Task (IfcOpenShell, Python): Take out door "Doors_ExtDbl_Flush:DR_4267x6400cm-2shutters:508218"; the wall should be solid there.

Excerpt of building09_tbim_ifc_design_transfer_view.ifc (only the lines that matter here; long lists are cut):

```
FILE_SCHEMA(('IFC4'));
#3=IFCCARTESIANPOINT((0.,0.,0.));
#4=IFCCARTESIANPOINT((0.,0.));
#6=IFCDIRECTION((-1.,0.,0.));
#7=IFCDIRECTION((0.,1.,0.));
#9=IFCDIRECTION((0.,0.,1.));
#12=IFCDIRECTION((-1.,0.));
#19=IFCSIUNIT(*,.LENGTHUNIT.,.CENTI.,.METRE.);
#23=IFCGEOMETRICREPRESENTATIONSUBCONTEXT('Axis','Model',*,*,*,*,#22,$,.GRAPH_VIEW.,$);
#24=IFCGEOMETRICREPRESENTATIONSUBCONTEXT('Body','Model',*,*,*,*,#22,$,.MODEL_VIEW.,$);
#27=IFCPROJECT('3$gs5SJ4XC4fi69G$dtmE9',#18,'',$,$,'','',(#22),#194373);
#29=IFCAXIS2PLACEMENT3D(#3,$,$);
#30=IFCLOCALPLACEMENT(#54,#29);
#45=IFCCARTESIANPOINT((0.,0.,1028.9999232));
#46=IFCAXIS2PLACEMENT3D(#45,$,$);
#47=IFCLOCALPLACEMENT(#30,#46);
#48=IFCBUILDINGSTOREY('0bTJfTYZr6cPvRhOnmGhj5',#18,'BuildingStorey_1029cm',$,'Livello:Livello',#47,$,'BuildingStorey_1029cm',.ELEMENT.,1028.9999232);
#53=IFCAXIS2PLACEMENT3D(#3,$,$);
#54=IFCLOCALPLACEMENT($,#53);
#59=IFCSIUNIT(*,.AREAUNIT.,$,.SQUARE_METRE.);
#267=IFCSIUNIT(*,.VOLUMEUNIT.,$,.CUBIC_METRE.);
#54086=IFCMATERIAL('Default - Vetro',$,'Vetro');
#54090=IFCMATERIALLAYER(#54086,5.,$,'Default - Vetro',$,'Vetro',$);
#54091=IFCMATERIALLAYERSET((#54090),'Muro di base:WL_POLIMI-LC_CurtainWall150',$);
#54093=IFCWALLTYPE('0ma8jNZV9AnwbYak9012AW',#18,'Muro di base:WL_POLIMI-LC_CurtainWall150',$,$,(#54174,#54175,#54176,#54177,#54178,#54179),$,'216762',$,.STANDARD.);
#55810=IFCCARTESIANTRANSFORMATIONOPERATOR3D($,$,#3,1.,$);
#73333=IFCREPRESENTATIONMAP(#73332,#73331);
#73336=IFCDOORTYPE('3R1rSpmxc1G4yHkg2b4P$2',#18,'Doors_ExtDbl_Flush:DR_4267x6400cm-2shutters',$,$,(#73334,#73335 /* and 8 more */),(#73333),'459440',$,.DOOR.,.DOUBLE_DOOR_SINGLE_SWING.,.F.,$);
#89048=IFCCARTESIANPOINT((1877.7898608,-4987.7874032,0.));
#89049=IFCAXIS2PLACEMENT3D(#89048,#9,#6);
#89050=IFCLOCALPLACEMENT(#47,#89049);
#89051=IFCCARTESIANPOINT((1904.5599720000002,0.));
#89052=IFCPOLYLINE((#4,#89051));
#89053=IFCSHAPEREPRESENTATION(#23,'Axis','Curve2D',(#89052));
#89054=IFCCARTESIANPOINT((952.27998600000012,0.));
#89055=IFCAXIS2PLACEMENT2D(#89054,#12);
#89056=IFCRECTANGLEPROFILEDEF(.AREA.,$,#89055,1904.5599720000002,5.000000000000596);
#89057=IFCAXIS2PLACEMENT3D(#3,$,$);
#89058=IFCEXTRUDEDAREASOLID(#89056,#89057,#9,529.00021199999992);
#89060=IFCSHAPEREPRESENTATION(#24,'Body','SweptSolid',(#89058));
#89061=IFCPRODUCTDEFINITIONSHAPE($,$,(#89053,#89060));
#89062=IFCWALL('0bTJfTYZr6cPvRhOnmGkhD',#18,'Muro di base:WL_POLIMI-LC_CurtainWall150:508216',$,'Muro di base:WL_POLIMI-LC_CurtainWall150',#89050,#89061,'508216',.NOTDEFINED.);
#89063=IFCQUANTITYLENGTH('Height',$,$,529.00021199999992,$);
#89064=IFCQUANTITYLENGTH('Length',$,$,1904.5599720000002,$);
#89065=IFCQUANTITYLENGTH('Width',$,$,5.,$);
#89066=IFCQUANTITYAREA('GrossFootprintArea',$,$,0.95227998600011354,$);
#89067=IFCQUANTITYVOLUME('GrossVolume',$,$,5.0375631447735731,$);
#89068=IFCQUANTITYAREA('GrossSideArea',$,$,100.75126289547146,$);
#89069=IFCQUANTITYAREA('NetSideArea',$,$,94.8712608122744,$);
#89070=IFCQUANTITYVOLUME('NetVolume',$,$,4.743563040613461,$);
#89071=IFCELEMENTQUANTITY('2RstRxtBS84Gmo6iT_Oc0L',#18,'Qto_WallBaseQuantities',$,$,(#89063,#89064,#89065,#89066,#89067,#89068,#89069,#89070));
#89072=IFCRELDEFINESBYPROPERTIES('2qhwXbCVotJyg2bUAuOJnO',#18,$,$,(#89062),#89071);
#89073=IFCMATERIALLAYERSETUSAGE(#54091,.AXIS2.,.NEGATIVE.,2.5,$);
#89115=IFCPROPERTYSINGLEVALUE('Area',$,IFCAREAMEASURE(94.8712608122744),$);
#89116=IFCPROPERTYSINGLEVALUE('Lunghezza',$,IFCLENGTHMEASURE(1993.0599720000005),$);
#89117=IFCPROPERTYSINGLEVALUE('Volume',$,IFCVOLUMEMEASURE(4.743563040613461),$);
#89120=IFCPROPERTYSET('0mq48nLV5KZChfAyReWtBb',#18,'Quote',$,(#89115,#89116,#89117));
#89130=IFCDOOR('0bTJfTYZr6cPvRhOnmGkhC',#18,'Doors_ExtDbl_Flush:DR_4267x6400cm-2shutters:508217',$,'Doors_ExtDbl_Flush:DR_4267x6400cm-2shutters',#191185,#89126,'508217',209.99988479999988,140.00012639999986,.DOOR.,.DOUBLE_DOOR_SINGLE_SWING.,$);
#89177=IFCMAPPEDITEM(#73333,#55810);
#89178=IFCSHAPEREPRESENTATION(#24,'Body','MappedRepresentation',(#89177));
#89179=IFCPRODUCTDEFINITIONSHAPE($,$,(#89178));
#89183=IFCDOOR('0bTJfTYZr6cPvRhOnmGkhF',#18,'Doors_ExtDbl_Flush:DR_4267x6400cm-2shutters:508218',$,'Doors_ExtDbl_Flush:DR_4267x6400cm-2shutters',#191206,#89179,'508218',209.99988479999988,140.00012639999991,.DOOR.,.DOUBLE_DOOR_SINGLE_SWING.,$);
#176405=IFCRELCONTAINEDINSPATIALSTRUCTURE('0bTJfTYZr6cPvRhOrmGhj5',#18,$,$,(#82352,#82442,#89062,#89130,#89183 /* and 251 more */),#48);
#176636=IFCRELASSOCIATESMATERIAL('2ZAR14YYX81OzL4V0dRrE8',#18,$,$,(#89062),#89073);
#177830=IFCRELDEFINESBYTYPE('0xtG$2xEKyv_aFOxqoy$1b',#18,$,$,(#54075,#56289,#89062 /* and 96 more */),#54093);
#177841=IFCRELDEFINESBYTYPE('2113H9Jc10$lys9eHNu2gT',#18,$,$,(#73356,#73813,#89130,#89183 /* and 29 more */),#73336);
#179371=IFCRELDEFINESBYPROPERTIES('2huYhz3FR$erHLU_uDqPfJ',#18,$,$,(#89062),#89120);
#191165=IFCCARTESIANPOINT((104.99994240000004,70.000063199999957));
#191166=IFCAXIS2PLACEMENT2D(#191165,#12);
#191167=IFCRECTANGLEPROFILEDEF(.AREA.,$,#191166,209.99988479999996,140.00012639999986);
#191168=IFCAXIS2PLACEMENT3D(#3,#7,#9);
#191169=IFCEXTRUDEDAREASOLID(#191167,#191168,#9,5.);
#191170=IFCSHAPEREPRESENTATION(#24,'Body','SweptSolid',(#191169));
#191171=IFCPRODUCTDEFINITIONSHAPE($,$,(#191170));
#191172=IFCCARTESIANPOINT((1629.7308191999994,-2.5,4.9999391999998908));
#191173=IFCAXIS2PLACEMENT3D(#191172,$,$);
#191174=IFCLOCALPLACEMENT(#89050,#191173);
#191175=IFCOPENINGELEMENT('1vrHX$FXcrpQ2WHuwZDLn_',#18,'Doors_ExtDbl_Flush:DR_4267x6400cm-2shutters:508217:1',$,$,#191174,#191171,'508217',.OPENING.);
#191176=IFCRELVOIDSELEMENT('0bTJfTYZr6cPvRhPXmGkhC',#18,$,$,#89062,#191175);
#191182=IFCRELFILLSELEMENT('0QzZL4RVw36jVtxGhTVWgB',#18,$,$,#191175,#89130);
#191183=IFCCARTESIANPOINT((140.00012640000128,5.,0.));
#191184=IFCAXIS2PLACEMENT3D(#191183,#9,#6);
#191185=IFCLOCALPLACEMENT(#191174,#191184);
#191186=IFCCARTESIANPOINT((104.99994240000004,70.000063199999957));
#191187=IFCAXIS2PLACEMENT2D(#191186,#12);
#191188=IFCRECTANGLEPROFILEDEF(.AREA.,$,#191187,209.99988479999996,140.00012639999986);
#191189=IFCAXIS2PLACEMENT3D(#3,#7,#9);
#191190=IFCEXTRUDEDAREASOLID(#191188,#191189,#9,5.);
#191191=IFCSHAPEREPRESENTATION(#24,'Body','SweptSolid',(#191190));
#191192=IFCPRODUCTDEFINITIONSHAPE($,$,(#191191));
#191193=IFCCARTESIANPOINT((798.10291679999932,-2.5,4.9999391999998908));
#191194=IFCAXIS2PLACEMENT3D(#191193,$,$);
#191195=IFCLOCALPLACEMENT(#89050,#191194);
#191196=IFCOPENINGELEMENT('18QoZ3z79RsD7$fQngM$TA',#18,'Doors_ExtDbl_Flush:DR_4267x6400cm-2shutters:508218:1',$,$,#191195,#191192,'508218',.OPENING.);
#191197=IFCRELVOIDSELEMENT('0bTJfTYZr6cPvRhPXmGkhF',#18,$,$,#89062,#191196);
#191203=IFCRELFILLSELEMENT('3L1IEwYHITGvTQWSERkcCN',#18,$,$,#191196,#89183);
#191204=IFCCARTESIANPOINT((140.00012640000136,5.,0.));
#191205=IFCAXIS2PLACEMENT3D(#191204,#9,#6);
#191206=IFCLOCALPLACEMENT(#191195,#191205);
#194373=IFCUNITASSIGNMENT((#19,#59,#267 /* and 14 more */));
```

```python
import ifcopenshell
import ifcopenshell.api.feature
import ifcopenshell.api.pset
import ifcopenshell.api.root
import ifcopenshell.geom
import ifcopenshell.util.element
import ifcopenshell.util.shape
import ifcopenshell.util.unit

model = ifcopenshell.open("building09_tbim_ifc_design_transfer_view.ifc")
area_scale = ifcopenshell.util.unit.calculate_unit_scale(model, "AREAUNIT")
volume_scale = ifcopenshell.util.unit.calculate_unit_scale(model, "VOLUMEUNIT")
settings = ifcopenshell.geom.settings()


def volume(element):
    """Net volume in cubic metres, openings subtracted."""
    shape = ifcopenshell.geom.create_shape(settings, element)
    return ifcopenshell.util.shape.get_volume(shape.geometry)


door = model.by_id(89183)
opening = door.FillsVoids[0].RelatingOpeningElement
wall = opening.VoidsElements[0].RelatingBuildingElement
before = volume(wall)

ifcopenshell.api.root.remove_product(model, product=door)
ifcopenshell.api.feature.remove_feature(model, feature=opening)

after = volume(wall)
thickness = 0.05  # wall thickness in metres

# Update the wall's stored quantities.
qto = model.by_id(ifcopenshell.util.element.get_pset(wall, "Qto_WallBaseQuantities", should_inherit=False)["id"])
ifcopenshell.api.pset.edit_qto(model, qto=qto, properties={
    "NetSideArea": after / thickness / area_scale,
    "NetVolume": after / volume_scale,
})
pset = model.by_id(ifcopenshell.util.element.get_pset(wall, "Quote", should_inherit=False)["id"])
ifcopenshell.api.pset.edit_pset(model, pset=pset, properties={
    "Area": model.create_entity("IfcAreaMeasure", after / thickness / area_scale),
    "Volume": model.create_entity("IfcVolumeMeasure", after / volume_scale),
})

print(f"wall volume {before:.3f} -> {after:.3f} m3")

model.write("building09_tbim_ifc_design_transfer_view-out.ifc")
```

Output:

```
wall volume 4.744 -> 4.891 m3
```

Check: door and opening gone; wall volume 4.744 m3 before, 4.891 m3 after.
